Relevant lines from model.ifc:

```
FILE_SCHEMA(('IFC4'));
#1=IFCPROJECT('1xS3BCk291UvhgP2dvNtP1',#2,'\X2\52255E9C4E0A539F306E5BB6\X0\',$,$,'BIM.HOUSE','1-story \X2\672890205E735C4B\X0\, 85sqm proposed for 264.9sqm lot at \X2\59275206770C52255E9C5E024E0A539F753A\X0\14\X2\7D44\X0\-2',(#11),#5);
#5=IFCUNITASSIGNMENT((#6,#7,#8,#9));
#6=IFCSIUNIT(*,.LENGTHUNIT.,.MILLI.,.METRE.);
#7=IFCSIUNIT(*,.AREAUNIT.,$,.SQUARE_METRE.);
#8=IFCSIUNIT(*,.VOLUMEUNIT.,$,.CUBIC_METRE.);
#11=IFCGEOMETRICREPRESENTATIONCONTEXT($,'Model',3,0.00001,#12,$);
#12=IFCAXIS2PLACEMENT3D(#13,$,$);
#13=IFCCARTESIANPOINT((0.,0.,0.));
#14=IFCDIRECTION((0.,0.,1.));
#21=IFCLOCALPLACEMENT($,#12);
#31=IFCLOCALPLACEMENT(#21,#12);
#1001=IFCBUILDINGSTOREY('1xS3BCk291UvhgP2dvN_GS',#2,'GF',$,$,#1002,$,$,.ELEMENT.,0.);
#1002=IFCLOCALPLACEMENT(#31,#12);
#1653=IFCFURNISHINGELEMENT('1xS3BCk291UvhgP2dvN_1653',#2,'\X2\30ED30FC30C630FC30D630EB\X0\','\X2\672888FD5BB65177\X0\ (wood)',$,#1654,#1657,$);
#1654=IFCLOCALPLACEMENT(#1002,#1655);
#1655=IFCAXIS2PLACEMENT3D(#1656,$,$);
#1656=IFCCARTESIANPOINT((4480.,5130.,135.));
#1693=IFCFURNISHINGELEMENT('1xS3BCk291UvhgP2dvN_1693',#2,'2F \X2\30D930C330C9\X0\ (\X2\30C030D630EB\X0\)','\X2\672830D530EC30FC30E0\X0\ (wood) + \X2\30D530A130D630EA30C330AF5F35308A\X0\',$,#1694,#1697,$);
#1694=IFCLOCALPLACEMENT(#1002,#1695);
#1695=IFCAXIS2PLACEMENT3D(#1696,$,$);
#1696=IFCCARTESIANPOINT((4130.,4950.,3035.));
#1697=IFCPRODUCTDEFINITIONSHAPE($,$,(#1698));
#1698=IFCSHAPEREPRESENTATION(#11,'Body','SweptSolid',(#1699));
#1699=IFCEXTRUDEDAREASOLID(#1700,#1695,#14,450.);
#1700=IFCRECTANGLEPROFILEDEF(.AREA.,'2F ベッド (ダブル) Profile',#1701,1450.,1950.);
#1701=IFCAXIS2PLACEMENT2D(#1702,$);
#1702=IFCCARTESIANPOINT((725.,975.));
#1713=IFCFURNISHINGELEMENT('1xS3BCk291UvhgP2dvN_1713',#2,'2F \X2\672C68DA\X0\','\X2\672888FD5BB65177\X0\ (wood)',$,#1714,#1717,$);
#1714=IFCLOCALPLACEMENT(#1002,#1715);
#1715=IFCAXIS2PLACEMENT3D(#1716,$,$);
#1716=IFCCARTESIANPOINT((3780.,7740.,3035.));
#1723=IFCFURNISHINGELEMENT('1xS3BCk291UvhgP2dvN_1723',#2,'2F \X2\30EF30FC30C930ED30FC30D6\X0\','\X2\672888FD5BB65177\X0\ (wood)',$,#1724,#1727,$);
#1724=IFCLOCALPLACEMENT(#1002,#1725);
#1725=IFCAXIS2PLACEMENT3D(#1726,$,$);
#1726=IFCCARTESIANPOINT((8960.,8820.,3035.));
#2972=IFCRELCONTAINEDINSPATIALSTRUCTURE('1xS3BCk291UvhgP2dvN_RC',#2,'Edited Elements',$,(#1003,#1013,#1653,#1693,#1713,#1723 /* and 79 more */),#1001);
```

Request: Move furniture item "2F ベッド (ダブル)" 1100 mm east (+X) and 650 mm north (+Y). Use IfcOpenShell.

```python
import ifcopenshell
import ifcopenshell.api.geometry
import ifcopenshell.util.placement

model = ifcopenshell.open("model.ifc")

item = model.by_guid("1xS3BCk291UvhgP2dvN_1693")
matrix = ifcopenshell.util.placement.get_local_placement(item.ObjectPlacement)
matrix[0, 3] += 1100.0
matrix[1, 3] += 650.0
ifcopenshell.api.geometry.edit_object_placement(model, product=item, matrix=matrix, is_si=False)

print(ifcopenshell.util.placement.get_local_placement(item.ObjectPlacement).round(3) + 0.0)

model.write("model_rev.ifc")
```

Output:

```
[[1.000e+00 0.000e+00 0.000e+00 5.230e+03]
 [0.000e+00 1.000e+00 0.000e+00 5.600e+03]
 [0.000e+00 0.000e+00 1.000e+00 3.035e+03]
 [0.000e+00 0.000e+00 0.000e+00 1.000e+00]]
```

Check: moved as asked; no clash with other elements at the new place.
